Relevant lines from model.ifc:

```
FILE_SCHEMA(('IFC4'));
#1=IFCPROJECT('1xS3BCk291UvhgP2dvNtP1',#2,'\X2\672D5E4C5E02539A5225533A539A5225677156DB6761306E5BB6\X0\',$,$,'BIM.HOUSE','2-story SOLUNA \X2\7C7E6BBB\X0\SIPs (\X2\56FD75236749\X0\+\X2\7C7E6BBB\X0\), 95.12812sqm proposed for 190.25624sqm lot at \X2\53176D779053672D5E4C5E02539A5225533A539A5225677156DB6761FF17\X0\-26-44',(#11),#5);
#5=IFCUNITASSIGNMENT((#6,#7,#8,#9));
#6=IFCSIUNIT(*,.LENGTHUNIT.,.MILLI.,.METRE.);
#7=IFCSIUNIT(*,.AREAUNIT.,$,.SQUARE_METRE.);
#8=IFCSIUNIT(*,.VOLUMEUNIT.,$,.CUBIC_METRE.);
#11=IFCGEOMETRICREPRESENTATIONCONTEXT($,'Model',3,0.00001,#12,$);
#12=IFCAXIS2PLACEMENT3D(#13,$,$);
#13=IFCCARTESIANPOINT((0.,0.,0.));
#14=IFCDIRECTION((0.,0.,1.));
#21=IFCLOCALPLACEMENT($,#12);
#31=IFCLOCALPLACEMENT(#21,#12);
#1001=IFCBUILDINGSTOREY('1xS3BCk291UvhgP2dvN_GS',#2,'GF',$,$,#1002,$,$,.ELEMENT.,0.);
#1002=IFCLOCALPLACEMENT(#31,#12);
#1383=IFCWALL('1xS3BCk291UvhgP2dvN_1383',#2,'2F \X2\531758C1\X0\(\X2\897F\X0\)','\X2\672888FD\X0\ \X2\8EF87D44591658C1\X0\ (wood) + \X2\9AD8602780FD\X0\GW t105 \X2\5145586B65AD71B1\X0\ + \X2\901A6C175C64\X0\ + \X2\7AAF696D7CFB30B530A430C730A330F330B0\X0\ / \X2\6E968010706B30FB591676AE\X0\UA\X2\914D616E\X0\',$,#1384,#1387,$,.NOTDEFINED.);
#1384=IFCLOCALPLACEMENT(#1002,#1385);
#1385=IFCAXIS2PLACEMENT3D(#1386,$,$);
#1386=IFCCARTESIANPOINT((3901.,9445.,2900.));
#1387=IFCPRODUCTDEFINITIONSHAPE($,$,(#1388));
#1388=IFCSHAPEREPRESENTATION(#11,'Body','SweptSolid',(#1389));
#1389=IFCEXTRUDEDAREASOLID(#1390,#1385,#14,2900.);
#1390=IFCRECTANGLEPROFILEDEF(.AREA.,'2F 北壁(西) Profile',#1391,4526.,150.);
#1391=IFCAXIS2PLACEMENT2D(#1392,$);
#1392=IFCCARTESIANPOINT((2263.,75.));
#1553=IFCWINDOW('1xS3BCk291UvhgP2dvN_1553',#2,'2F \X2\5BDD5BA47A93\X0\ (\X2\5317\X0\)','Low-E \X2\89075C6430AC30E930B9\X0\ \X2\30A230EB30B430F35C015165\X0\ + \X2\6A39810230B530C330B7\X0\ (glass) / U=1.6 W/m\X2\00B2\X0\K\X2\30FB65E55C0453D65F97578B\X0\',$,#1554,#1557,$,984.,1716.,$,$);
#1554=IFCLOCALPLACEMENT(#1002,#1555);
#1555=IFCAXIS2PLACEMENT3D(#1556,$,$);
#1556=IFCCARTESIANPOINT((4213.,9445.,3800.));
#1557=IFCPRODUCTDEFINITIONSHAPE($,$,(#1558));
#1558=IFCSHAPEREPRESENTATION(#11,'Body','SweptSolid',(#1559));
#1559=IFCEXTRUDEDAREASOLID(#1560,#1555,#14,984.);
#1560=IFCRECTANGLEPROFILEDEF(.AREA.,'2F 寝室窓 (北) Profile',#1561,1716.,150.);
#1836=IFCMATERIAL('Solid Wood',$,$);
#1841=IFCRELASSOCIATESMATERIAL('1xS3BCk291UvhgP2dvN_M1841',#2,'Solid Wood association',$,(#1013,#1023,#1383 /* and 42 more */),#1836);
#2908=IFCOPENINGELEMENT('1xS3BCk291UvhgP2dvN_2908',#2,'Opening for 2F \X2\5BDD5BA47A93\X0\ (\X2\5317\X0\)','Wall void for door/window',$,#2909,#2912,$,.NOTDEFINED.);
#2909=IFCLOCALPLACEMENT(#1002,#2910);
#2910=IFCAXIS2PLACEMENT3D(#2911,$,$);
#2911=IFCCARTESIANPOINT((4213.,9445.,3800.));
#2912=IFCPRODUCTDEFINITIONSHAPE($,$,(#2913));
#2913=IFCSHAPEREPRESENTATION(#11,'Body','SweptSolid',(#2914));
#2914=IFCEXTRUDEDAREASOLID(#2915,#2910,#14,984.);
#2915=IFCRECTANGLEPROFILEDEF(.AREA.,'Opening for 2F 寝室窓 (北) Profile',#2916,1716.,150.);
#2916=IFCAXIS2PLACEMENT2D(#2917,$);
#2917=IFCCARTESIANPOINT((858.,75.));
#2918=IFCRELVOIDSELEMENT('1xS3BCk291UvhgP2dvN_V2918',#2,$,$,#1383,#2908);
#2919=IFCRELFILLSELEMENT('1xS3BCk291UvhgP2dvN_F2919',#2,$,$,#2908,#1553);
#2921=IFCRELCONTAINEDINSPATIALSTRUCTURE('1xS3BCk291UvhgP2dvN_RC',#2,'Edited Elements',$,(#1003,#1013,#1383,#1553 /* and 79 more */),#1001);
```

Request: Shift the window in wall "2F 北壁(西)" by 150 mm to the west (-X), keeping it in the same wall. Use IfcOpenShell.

```python
import ifcopenshell
import ifcopenshell.api.geometry
import ifcopenshell.util.placement
import ifcopenshell.util.unit

model = ifcopenshell.open("model.ifc")
unit_scale = ifcopenshell.util.unit.calculate_unit_scale(model)

window = model.by_guid("1xS3BCk291UvhgP2dvN_1553")
opening = window.FillsVoids[0].RelatingOpeningElement
wall = opening.VoidsElements[0].RelatingBuildingElement

wall_matrix = ifcopenshell.util.placement.get_local_placement(wall.ObjectPlacement)
shift = wall_matrix[:3, 0] * -0.15 / unit_scale
before = ifcopenshell.util.placement.get_local_placement(window.ObjectPlacement)[:3, 3].copy()

# The window is not placed relative to its opening, so move both.
for product in (opening, window):
    matrix = ifcopenshell.util.placement.get_local_placement(product.ObjectPlacement)
    matrix[:3, 3] += shift
    ifcopenshell.api.geometry.edit_object_placement(model, product=product, matrix=matrix, is_si=False)

after = ifcopenshell.util.placement.get_local_placement(window.ObjectPlacement)[:3, 3]
print("window moved by", (after - before).round(3) + 0.0)

model.write("model_edited.ifc")
```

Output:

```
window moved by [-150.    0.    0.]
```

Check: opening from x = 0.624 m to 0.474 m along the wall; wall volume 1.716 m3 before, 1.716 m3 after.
